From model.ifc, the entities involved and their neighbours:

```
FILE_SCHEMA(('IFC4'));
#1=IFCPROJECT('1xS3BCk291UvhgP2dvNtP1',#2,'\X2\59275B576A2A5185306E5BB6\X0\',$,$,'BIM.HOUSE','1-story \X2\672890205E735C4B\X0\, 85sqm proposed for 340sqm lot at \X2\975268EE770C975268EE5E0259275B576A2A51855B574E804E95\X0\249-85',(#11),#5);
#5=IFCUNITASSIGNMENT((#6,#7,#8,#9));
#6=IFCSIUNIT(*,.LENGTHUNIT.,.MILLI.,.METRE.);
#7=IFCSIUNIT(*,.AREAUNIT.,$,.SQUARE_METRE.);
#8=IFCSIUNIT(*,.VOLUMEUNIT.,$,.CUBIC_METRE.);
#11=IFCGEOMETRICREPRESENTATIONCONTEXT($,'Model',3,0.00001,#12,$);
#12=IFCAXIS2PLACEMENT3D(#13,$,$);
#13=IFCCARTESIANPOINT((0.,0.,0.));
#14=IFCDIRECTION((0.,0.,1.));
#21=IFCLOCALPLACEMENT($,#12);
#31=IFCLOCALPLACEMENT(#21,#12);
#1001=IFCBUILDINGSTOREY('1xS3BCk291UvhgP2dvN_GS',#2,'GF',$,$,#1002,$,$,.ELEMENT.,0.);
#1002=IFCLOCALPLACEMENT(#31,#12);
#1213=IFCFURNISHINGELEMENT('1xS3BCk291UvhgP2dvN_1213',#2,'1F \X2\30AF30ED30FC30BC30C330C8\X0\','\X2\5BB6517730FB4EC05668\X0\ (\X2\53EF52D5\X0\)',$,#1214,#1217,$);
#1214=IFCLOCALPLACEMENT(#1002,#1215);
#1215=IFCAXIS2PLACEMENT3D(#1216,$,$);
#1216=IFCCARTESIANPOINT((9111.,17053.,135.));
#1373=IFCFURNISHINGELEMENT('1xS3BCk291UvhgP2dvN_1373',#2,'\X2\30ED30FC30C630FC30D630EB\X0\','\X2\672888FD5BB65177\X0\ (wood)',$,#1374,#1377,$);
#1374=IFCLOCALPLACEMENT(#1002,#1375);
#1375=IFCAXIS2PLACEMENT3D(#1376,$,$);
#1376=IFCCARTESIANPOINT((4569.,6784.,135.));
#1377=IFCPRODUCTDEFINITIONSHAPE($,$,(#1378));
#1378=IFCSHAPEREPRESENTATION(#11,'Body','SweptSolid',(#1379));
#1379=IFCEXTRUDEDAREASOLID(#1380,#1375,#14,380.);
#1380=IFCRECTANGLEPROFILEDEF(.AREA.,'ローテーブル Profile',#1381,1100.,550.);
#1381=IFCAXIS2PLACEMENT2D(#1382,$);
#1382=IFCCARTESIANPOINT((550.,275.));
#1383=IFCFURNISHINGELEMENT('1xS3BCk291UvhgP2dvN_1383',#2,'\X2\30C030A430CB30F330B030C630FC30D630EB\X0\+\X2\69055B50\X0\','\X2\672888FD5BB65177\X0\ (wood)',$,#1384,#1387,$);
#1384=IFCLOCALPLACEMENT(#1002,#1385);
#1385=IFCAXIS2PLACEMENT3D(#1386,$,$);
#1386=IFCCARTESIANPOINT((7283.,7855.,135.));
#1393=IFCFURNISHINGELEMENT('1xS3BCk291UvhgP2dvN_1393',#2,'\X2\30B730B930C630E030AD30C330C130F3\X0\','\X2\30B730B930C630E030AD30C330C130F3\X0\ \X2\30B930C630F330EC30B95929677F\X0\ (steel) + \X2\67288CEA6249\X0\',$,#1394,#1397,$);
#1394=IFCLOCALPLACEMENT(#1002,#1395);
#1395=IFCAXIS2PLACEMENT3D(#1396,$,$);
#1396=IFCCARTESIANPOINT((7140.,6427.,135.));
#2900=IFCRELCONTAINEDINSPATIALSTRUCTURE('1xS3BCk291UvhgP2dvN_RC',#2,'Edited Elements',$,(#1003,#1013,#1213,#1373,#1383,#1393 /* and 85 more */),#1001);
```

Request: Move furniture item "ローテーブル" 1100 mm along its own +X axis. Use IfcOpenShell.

```python
import ifcopenshell
import ifcopenshell.api.geometry
import ifcopenshell.util.placement

model = ifcopenshell.open("model.ifc")

item = model.by_id(1373)
matrix = ifcopenshell.util.placement.get_local_placement(item.ObjectPlacement)
matrix[:3, 3] += matrix[:3, 0] * 1100.0
ifcopenshell.api.geometry.edit_object_placement(model, product=item, matrix=matrix, is_si=False)

print(ifcopenshell.util.placement.get_local_placement(item.ObjectPlacement).round(3) + 0.0)

model.write("model-out.ifc")
```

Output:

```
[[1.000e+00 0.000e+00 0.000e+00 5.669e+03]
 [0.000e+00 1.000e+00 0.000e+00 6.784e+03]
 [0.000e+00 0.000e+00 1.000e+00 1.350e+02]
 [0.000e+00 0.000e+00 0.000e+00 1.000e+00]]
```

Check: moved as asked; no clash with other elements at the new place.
